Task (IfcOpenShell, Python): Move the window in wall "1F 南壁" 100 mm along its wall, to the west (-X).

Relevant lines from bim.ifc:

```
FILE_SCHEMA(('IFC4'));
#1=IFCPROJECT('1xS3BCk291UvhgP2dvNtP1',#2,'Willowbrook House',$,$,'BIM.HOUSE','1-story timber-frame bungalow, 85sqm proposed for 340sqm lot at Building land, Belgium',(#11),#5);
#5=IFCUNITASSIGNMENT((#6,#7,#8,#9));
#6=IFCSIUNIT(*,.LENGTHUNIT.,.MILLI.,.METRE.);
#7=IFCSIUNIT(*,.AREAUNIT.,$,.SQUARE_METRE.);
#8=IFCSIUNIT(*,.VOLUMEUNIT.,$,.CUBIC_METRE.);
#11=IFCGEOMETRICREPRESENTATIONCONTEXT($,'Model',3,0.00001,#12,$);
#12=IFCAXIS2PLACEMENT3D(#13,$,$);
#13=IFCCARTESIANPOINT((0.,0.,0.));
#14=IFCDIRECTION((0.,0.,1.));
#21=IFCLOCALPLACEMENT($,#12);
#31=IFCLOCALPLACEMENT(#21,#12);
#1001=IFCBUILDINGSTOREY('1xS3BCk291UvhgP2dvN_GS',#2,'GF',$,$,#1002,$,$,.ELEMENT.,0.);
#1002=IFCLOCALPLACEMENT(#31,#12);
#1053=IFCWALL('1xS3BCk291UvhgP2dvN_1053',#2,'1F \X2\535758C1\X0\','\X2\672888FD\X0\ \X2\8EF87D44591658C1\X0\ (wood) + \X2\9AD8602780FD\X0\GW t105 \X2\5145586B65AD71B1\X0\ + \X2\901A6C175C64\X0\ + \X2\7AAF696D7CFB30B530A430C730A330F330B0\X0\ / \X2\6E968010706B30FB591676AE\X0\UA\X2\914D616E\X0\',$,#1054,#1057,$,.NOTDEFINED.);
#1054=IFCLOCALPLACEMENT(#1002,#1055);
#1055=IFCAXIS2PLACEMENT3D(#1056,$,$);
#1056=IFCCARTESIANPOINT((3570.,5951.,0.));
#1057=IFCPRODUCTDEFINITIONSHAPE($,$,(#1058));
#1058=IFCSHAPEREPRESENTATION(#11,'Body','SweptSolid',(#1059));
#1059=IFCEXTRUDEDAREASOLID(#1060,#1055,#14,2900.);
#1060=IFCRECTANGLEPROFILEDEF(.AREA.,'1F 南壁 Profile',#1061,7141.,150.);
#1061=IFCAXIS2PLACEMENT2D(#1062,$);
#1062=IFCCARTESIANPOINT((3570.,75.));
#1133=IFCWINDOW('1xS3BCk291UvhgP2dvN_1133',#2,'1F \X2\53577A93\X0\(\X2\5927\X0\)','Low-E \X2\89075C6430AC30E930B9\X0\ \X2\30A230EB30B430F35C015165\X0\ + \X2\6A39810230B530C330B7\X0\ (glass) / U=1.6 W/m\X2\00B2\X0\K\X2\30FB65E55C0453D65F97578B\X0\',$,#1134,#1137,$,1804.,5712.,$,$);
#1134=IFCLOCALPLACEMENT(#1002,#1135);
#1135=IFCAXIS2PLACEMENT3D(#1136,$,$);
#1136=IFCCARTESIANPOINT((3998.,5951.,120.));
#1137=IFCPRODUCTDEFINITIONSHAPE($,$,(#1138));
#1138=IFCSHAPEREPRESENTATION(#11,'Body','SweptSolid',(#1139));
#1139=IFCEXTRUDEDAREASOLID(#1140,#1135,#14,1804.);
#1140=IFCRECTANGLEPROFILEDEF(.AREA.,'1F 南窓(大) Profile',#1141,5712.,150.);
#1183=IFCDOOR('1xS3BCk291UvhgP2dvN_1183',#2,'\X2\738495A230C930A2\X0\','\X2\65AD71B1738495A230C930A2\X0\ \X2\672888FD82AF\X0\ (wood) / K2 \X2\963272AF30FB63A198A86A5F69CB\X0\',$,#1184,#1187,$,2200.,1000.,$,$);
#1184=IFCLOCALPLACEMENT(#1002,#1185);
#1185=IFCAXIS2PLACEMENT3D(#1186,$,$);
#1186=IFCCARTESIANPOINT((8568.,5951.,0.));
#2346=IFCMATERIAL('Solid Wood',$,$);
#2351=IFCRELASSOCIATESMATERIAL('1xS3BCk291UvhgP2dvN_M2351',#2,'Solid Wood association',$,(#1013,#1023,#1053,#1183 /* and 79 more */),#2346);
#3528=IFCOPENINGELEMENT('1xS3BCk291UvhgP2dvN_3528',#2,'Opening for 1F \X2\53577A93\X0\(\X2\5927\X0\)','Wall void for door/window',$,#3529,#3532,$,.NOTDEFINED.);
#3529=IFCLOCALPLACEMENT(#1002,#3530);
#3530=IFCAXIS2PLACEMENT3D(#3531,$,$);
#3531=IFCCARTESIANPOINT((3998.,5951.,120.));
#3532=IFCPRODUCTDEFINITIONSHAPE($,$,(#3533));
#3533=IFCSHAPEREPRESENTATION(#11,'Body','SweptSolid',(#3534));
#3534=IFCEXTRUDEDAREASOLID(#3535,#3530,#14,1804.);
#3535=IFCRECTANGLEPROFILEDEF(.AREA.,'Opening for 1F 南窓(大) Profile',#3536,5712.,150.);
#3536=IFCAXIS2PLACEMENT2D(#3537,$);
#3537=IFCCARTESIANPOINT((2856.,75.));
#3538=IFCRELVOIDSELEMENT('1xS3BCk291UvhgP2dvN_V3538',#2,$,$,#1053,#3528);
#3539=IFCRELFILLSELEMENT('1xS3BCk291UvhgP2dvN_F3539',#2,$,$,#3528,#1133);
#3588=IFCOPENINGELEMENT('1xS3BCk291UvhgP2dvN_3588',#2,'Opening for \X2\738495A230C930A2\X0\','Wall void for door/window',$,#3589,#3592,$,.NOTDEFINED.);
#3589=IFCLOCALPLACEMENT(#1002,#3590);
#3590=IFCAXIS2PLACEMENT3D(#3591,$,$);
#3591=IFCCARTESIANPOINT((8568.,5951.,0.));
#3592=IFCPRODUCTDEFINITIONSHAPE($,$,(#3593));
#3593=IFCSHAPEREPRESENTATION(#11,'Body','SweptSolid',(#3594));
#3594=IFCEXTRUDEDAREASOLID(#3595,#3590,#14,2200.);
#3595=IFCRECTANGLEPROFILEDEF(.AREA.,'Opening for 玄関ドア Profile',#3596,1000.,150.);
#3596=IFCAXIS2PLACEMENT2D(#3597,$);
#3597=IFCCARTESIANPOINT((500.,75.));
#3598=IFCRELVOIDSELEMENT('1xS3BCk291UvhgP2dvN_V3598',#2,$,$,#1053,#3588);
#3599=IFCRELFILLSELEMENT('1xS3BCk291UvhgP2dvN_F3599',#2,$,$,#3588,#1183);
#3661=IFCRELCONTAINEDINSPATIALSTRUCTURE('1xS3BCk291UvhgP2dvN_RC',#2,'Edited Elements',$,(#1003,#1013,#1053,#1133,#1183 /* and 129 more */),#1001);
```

```python
import ifcopenshell
import ifcopenshell.api.geometry
import ifcopenshell.util.placement

model = ifcopenshell.open("bim.ifc")

window = model.by_id(1133)
opening = window.FillsVoids[0].RelatingOpeningElement
wall = opening.VoidsElements[0].RelatingBuildingElement

wall_matrix = ifcopenshell.util.placement.get_local_placement(wall.ObjectPlacement)
shift = wall_matrix[:3, 0] * -100.0
before = ifcopenshell.util.placement.get_local_placement(window.ObjectPlacement)[:3, 3].copy()

# The window is not placed relative to its opening, so move both.
for product in (opening, window):
    matrix = ifcopenshell.util.placement.get_local_placement(product.ObjectPlacement)
    matrix[:3, 3] += shift
    ifcopenshell.api.geometry.edit_object_placement(model, product=product, matrix=matrix, is_si=False)

after = ifcopenshell.util.placement.get_local_placement(window.ObjectPlacement)[:3, 3]
print("window moved by", (after - before).round(3) + 0.0)

model.write("bim_updated.ifc")
```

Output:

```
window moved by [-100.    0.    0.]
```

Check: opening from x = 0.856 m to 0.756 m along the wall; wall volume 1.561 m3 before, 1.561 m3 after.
